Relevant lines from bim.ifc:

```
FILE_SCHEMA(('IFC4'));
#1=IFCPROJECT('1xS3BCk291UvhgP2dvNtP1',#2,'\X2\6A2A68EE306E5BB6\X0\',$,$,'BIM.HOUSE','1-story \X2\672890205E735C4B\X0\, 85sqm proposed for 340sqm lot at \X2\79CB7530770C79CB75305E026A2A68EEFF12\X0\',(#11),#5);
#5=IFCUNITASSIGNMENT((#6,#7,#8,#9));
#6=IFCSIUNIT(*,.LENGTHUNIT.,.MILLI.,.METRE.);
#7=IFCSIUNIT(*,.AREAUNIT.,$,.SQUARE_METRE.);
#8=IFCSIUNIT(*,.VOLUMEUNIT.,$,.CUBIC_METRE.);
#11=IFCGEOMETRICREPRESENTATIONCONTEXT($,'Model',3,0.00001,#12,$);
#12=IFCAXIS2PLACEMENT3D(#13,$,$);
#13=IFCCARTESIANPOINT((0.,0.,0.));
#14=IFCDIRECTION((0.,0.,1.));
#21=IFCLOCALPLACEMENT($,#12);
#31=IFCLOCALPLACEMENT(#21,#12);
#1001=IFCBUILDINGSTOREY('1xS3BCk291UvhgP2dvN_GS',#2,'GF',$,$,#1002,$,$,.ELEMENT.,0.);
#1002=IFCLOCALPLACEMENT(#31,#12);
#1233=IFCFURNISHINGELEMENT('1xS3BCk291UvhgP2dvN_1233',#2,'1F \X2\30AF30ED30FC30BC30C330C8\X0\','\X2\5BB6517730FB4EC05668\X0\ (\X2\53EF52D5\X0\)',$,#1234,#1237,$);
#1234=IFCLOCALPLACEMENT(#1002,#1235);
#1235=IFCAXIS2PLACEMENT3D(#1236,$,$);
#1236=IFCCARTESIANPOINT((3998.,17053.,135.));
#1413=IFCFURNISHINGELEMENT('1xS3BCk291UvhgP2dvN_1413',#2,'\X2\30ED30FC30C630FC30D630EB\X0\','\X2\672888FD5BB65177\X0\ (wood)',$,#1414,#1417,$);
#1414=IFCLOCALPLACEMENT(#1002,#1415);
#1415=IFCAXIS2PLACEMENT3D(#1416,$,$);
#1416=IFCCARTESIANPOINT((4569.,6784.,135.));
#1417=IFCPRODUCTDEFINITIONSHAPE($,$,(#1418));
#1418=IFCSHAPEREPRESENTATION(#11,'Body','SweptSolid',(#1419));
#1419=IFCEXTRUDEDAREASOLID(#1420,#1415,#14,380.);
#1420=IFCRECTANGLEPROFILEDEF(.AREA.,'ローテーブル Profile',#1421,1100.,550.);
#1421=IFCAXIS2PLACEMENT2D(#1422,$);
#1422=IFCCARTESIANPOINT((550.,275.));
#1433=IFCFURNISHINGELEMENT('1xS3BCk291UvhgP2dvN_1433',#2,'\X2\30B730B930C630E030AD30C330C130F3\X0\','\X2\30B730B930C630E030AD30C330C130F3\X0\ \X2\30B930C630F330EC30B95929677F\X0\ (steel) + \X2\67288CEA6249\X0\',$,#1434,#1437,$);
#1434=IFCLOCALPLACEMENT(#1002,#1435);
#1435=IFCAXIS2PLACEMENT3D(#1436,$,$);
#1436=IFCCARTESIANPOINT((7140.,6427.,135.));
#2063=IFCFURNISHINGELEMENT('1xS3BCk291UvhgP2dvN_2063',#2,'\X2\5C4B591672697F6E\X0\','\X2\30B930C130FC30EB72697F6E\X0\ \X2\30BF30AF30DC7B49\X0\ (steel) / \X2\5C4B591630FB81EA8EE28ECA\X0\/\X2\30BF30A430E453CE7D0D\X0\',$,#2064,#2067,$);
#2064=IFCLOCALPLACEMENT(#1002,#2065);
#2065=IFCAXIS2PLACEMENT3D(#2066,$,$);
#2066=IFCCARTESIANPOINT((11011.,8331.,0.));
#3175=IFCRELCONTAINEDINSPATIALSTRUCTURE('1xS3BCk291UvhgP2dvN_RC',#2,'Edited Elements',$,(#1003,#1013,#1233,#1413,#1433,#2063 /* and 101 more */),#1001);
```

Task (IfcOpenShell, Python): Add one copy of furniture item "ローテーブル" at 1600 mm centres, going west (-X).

```python
import numpy as np
import ifcopenshell
import ifcopenshell.api.geometry
import ifcopenshell.api.root
import ifcopenshell.util.element
import ifcopenshell.util.placement
import ifcopenshell.util.unit

model = ifcopenshell.open("bim.ifc")
unit_scale = ifcopenshell.util.unit.calculate_unit_scale(model)


def reuse_history(source, copy):
    """copy_class also copies each property set's owner history, people and application; keep the originals."""
    for rel in copy.IsDefinedBy:
        if rel.is_a("IfcRelDefinesByProperties") and (history := rel.RelatingPropertyDefinition.OwnerHistory):
            rel.RelatingPropertyDefinition.OwnerHistory = source.OwnerHistory
            ifcopenshell.util.element.remove_deep2(model, history)


source = model.by_guid("1xS3BCk291UvhgP2dvN_1413")
base = ifcopenshell.util.placement.get_local_placement(source.ObjectPlacement)
step = np.array([-1.0, 0.0, 0.0]) * 1.6 / unit_scale

for i in range(1, 2):
    copy = ifcopenshell.api.root.copy_class(model, product=source)
    copy.Representation = ifcopenshell.util.element.copy_deep(
        model, source.Representation, exclude=["IfcGeometricRepresentationContext", "IfcRepresentationMap"]
    )
    reuse_history(source, copy)
    matrix = base.copy()
    matrix[:3, 3] += i * step
    print("added at", matrix[:3, 3].round(3) + 0.0)
    ifcopenshell.api.geometry.edit_object_placement(model, product=copy, matrix=matrix, is_si=False)

model.write("bim_updated.ifc")
```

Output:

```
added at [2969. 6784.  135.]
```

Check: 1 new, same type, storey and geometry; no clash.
